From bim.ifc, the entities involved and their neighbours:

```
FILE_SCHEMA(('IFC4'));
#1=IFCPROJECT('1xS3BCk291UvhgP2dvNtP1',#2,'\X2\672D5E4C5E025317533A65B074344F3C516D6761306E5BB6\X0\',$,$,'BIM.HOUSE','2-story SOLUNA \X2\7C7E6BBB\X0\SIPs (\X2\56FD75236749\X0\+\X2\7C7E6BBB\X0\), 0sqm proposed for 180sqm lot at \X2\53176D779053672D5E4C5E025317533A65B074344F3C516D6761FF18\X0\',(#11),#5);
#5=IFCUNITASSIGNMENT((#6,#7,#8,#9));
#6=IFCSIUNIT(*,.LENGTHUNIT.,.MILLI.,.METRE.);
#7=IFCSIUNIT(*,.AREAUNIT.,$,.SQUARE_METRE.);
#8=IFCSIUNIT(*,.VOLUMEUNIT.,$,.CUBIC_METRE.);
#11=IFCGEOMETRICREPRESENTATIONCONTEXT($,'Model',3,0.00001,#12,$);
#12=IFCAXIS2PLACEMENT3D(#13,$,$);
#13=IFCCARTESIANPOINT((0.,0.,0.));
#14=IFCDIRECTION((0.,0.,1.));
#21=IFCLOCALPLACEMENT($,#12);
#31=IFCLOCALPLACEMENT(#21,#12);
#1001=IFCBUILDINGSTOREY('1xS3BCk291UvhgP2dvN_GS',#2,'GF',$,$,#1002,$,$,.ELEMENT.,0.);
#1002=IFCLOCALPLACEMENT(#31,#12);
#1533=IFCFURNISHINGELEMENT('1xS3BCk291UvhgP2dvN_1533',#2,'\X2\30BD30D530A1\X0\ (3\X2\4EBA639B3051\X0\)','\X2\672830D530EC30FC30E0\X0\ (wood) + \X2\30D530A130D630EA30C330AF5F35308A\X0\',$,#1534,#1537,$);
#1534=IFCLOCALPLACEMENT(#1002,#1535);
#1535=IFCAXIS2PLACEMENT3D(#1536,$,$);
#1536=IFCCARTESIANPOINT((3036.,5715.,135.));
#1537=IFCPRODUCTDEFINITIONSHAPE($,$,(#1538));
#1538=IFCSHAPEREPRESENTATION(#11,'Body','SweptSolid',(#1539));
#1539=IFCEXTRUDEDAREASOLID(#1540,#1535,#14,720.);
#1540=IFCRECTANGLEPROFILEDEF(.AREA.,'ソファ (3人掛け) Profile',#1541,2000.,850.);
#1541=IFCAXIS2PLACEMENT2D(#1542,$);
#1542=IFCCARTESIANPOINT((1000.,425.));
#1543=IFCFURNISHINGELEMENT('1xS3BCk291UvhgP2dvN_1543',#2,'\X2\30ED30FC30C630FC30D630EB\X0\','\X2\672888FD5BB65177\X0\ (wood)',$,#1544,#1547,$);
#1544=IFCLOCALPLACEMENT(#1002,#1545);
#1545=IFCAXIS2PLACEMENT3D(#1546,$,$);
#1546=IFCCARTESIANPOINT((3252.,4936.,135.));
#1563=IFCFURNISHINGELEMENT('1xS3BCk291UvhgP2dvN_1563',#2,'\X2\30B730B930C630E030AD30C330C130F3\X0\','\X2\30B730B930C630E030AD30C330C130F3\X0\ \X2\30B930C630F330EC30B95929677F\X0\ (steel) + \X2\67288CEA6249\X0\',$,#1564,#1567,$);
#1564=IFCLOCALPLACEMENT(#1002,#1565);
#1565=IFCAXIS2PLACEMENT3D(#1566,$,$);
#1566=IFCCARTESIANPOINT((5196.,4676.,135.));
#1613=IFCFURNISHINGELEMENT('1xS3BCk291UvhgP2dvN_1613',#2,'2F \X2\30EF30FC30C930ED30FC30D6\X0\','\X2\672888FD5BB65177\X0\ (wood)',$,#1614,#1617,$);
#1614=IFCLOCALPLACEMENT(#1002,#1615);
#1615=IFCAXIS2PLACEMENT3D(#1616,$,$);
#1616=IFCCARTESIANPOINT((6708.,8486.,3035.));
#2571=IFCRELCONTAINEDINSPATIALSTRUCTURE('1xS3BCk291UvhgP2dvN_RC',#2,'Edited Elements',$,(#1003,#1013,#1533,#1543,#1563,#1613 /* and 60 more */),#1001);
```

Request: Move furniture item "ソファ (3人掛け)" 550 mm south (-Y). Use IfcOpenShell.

```python
import ifcopenshell
import ifcopenshell.api.geometry
import ifcopenshell.util.placement
import ifcopenshell.util.unit

model = ifcopenshell.open("bim.ifc")
unit_scale = ifcopenshell.util.unit.calculate_unit_scale(model)

item = model.by_id(1533)
matrix = ifcopenshell.util.placement.get_local_placement(item.ObjectPlacement)
matrix[1, 3] -= 0.55 / unit_scale
ifcopenshell.api.geometry.edit_object_placement(model, product=item, matrix=matrix, is_si=False)

print(ifcopenshell.util.placement.get_local_placement(item.ObjectPlacement).round(3) + 0.0)

model.write("bim_rev.ifc")
```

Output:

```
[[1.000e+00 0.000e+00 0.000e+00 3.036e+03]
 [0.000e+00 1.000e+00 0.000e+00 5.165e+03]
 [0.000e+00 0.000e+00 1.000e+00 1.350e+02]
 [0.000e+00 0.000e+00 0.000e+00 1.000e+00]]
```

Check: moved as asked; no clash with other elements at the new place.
